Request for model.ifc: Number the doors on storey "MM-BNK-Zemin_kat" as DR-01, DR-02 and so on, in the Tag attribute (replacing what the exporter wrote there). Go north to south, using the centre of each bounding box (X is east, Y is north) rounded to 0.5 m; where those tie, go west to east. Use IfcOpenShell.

First a look at what the model holds.

```python
import ifcopenshell
import ifcopenshell.util.element
import ifcopenshell.util.placement

model = ifcopenshell.open("model.ifc")
print(model.schema)
storey = next(s for s in model.by_type("IfcBuildingStorey") if s.Name == "MM-BNK-Zemin_kat")
doors = [e for e in ifcopenshell.util.element.get_decomposition(storey) if e.is_a("IfcDoor")]
for e in sorted(doors, key=lambda e: e.id()):
    origin = ifcopenshell.util.placement.get_local_placement(e.ObjectPlacement)[:3, 3]
    print(e.id(), e.Tag, e.Name, origin.round(2) + 0.0, sep=" | ")
```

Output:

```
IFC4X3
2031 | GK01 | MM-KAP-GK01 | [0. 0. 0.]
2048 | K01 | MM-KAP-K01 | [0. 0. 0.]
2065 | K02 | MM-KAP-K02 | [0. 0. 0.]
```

```python
import ifcopenshell
import ifcopenshell.geom
import ifcopenshell.util.element
import ifcopenshell.util.shape

model = ifcopenshell.open("model.ifc")
settings = ifcopenshell.geom.settings()
settings.set("use-world-coords", True)


def centre(element):
    shape = ifcopenshell.geom.create_shape(settings, element)
    return ifcopenshell.util.shape.get_bbox_centroid(shape.geometry)


storey = next(s for s in model.by_type("IfcBuildingStorey") if s.Name == "MM-BNK-Zemin_kat")
doors = [e for e in ifcopenshell.util.element.get_decomposition(storey) if e.is_a("IfcDoor")]

# Insertion points can sit at a corner or the storey origin, so sort by the geometry (in metres).
centres = {e: centre(e) for e in doors}
doors.sort(key=lambda e: (-round(centres[e][1] / 0.5), centres[e][0]))

for i, e in enumerate(doors, start=1):
    number = f"DR-{i:02d}"
    e.Tag = number
    print(e.id(), number)

model.write("model-out.ifc")
```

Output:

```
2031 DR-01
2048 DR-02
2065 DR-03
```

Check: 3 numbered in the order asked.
